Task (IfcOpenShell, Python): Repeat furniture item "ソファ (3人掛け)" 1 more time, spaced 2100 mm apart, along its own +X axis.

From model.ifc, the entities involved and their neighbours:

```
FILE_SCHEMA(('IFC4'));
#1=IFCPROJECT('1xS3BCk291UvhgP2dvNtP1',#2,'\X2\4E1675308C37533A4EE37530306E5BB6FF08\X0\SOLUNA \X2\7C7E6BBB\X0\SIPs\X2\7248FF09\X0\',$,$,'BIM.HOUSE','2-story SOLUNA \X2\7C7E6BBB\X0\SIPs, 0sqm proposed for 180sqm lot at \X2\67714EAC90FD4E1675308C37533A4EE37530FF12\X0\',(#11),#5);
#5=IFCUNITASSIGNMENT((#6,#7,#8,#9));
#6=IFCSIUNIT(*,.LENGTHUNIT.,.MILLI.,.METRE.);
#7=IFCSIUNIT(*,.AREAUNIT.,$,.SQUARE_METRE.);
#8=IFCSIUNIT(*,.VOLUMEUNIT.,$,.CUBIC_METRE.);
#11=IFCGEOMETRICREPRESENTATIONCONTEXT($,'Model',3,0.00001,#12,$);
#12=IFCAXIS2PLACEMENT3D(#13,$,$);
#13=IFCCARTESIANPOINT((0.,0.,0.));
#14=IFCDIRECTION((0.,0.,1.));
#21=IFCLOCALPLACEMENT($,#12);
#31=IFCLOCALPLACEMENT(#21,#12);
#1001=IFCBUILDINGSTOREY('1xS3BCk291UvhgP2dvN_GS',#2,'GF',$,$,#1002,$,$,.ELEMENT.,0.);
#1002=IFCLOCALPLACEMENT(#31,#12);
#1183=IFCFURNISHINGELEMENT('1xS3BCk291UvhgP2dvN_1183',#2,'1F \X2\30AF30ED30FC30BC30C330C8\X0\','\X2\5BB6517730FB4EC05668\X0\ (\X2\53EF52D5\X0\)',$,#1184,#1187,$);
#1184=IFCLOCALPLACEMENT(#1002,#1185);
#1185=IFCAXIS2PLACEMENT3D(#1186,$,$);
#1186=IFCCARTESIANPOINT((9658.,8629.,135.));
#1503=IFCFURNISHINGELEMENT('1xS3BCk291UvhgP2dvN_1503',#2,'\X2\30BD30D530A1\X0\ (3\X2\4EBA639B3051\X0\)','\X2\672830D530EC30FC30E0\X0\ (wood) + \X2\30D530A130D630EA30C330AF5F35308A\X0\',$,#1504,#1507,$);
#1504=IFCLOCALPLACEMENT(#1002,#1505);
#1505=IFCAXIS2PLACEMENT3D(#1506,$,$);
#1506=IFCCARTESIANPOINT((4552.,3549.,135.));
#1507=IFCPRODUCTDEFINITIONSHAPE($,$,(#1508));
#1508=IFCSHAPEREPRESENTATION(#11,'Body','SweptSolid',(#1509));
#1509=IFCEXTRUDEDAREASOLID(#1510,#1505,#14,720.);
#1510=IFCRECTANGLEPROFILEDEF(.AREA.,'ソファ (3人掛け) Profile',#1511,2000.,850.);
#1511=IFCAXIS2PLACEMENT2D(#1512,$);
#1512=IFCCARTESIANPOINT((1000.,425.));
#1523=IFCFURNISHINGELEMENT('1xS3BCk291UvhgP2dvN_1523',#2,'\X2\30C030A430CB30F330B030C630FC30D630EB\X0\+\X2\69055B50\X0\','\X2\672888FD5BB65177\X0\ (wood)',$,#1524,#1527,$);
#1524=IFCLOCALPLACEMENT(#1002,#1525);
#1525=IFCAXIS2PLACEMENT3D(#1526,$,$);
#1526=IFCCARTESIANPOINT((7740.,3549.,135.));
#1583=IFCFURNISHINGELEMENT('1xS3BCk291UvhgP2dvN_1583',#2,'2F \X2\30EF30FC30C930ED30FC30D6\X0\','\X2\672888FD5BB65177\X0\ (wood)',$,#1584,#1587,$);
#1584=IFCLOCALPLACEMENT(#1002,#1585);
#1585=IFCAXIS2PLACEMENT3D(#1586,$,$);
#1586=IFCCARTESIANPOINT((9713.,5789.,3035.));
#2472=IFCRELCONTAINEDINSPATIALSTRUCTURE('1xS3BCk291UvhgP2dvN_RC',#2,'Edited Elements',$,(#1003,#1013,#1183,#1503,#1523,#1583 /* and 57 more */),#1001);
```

```python
import ifcopenshell
import ifcopenshell.api.geometry
import ifcopenshell.api.root
import ifcopenshell.util.element
import ifcopenshell.util.placement
import ifcopenshell.util.unit

model = ifcopenshell.open("model.ifc")
unit_scale = ifcopenshell.util.unit.calculate_unit_scale(model)


def reuse_history(source, copy):
    """copy_class also copies each property set's owner history, people and application; keep the originals."""
    for rel in copy.IsDefinedBy:
        if rel.is_a("IfcRelDefinesByProperties") and (history := rel.RelatingPropertyDefinition.OwnerHistory):
            rel.RelatingPropertyDefinition.OwnerHistory = source.OwnerHistory
            ifcopenshell.util.element.remove_deep2(model, history)


source = model.by_guid("1xS3BCk291UvhgP2dvN_1503")
base = ifcopenshell.util.placement.get_local_placement(source.ObjectPlacement)
step = base[:3, 0] * 2.1 / unit_scale

for i in range(1, 2):
    copy = ifcopenshell.api.root.copy_class(model, product=source)
    copy.Representation = ifcopenshell.util.element.copy_deep(
        model, source.Representation, exclude=["IfcGeometricRepresentationContext", "IfcRepresentationMap"]
    )
    reuse_history(source, copy)
    matrix = base.copy()
    matrix[:3, 3] += i * step
    print("added at", matrix[:3, 3].round(3) + 0.0)
    ifcopenshell.api.geometry.edit_object_placement(model, product=copy, matrix=matrix, is_si=False)

model.write("model_v2.ifc")
```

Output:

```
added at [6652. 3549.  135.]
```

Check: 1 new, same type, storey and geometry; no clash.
